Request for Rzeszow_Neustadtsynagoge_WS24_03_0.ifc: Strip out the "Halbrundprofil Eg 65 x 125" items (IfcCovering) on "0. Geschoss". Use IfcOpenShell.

First a look at what the model holds.

```python
import ifcopenshell
import ifcopenshell.util.element

model = ifcopenshell.open("Rzeszow_Neustadtsynagoge_WS24_03_0.ifc")
print(model.schema)
storey = next(s for s in model.by_type("IfcBuildingStorey") if s.Name == "0. Geschoss")
coverings = [e for e in ifcopenshell.util.element.get_decomposition(storey) if e.is_a("IfcCovering")]
seen = {}
for e in coverings:
    element_type = ifcopenshell.util.element.get_type(e)
    name = element_type.Name if element_type not in (None, e) else None
    seen[name] = seen.get(name, 0) + 1
for name, count in sorted(seen.items(), key=str):
    print(count, "x", name)
```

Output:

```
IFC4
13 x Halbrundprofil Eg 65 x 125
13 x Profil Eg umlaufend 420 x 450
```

```python
import ifcopenshell
import ifcopenshell.api.root
import ifcopenshell.util.element

model = ifcopenshell.open("Rzeszow_Neustadtsynagoge_WS24_03_0.ifc")

storey = next(s for s in model.by_type("IfcBuildingStorey") if s.Name == "0. Geschoss")
coverings = [e for e in ifcopenshell.util.element.get_decomposition(storey) if e.is_a("IfcCovering")]
targets = [e for e in coverings if (t := ifcopenshell.util.element.get_type(e)) not in (None, e) and t.Name == "Halbrundprofil Eg 65 x 125"]

for e in targets:
    ifcopenshell.api.root.remove_product(model, product=e)
print(len(targets), "removed")

model.write("Rzeszow_Neustadtsynagoge_WS24_03_0_rev.ifc")
```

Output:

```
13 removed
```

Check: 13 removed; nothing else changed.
